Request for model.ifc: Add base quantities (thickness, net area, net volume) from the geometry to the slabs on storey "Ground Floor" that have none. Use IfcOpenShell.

First a look at what the model holds.

```python
import ifcopenshell
import ifcopenshell.util.element
import ifcopenshell.util.unit

model = ifcopenshell.open("model.ifc")
print(model.schema)
for unit_type in ("LENGTHUNIT", "AREAUNIT", "VOLUMEUNIT"):
    print(unit_type, ifcopenshell.util.unit.calculate_unit_scale(model, unit_type))
storey = next(s for s in model.by_type("IfcBuildingStorey") if s.Name == "Ground Floor")
slabs = [e for e in ifcopenshell.util.element.get_decomposition(storey) if e.is_a("IfcSlab")]
for e in sorted(slabs, key=lambda e: e.id()):
    print(e.id(), e.is_a(), e.Name, list(ifcopenshell.util.element.get_psets(e, qtos_only=True)), sep=" | ")
```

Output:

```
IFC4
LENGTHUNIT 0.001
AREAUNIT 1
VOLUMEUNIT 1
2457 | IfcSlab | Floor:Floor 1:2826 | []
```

```python
import ifcopenshell
import ifcopenshell.api.pset
import ifcopenshell.geom
import ifcopenshell.util.element
import ifcopenshell.util.shape
import ifcopenshell.util.unit

model = ifcopenshell.open("model.ifc")
unit_scale = ifcopenshell.util.unit.calculate_unit_scale(model)
area_scale = ifcopenshell.util.unit.calculate_unit_scale(model, "AREAUNIT")
volume_scale = ifcopenshell.util.unit.calculate_unit_scale(model, "VOLUMEUNIT")
settings = ifcopenshell.geom.settings()

storey = next(s for s in model.by_type("IfcBuildingStorey") if s.Name == "Ground Floor")
slabs = [e for e in ifcopenshell.util.element.get_decomposition(storey) if e.is_a("IfcSlab")]

for e in sorted(slabs, key=lambda e: e.id()):
    if ifcopenshell.util.element.get_psets(e, qtos_only=True, should_inherit=False):
        continue
    # Geometry comes back in metres, in the element's own axes.
    shape = ifcopenshell.geom.create_shape(settings, e)
    values = {
        "Width": ifcopenshell.util.shape.get_z(shape.geometry) / unit_scale,
        "NetArea": ifcopenshell.util.shape.get_footprint_area(shape.geometry) / area_scale,
        "NetVolume": ifcopenshell.util.shape.get_volume(shape.geometry) / volume_scale,
    }
    qto = ifcopenshell.api.pset.add_qto(model, product=e, name="Qto_SlabBaseQuantities")
    ifcopenshell.api.pset.edit_qto(model, qto=qto, properties=values)
    print(e.id(), {k: round(v, 3) for k, v in values.items()})

model.write("model_rev.ifc")
```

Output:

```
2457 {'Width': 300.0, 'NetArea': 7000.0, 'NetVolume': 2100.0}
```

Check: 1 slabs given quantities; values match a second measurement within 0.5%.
